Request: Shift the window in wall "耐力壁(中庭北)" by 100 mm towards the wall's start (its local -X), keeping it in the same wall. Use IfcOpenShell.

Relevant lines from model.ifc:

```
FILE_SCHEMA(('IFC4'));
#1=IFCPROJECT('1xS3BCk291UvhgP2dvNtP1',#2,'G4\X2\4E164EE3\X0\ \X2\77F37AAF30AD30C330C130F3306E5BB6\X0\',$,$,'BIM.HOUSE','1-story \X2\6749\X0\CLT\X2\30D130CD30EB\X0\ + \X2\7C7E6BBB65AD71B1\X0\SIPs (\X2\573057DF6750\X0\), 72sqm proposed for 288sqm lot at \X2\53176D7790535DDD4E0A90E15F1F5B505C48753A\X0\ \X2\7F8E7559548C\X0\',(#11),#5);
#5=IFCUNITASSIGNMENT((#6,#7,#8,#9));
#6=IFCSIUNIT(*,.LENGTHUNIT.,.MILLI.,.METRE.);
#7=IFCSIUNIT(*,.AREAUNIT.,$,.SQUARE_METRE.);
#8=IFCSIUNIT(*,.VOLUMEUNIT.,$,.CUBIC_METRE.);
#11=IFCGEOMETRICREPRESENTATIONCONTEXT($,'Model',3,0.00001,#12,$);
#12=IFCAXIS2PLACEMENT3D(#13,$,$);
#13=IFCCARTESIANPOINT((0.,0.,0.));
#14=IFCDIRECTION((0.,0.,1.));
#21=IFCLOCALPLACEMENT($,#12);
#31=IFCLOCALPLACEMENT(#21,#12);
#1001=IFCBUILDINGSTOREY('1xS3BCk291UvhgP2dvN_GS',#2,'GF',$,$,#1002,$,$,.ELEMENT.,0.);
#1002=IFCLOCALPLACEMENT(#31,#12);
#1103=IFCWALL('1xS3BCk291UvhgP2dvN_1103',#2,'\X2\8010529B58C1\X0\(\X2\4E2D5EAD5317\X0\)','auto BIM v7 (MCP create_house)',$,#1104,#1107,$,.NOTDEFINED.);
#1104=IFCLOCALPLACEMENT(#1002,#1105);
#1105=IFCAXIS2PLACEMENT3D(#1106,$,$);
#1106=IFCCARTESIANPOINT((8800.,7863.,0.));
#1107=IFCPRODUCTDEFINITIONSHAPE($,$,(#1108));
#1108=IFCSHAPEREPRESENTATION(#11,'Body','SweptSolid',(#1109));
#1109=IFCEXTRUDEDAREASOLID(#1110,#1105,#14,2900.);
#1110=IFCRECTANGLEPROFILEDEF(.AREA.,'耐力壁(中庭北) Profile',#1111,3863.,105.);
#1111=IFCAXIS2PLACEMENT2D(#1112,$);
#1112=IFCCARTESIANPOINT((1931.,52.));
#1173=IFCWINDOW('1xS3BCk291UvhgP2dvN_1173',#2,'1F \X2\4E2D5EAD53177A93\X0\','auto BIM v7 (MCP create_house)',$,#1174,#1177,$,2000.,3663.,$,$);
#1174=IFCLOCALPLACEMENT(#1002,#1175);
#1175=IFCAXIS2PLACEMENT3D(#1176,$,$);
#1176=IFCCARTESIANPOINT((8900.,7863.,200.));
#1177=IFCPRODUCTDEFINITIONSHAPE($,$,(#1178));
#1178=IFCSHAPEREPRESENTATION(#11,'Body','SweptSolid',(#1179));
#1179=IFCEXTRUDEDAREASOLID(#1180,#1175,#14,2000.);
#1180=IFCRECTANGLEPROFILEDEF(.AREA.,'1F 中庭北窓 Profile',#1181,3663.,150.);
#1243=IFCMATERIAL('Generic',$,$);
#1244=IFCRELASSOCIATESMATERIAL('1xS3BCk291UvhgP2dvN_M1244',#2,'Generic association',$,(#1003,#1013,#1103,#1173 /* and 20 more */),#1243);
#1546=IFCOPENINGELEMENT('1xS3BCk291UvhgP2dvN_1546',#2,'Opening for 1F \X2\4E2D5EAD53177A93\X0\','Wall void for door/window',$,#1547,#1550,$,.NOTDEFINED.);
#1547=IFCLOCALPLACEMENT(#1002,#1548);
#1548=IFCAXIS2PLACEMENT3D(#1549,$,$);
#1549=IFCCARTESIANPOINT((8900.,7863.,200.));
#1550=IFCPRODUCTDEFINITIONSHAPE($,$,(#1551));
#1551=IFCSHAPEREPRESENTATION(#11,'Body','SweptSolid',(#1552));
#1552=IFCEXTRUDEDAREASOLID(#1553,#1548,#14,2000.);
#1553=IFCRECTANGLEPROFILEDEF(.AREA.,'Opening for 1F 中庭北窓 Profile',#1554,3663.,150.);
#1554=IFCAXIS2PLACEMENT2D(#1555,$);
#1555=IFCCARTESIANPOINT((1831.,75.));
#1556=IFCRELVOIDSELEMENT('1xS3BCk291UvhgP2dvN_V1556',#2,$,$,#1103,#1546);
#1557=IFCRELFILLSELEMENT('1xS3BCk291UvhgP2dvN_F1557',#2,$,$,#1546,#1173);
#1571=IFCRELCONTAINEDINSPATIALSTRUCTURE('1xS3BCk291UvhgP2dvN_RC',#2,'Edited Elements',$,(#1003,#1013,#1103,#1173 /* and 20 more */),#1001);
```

```python
import ifcopenshell
import ifcopenshell.api.geometry
import ifcopenshell.util.placement
import ifcopenshell.util.unit

model = ifcopenshell.open("model.ifc")
unit_scale = ifcopenshell.util.unit.calculate_unit_scale(model)

window = model.by_id(1173)
opening = window.FillsVoids[0].RelatingOpeningElement
wall = opening.VoidsElements[0].RelatingBuildingElement

wall_matrix = ifcopenshell.util.placement.get_local_placement(wall.ObjectPlacement)
shift = wall_matrix[:3, 0] * -0.1 / unit_scale
before = ifcopenshell.util.placement.get_local_placement(window.ObjectPlacement)[:3, 3].copy()

# The window is not placed relative to its opening, so move both.
for product in (opening, window):
    matrix = ifcopenshell.util.placement.get_local_placement(product.ObjectPlacement)
    matrix[:3, 3] += shift
    ifcopenshell.api.geometry.edit_object_placement(model, product=product, matrix=matrix, is_si=False)

after = ifcopenshell.util.placement.get_local_placement(window.ObjectPlacement)[:3, 3]
print("window moved by", (after - before).round(3) + 0.0)

model.write("model_rev.ifc")
```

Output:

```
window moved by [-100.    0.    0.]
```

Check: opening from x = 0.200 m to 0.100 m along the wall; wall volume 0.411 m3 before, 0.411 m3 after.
